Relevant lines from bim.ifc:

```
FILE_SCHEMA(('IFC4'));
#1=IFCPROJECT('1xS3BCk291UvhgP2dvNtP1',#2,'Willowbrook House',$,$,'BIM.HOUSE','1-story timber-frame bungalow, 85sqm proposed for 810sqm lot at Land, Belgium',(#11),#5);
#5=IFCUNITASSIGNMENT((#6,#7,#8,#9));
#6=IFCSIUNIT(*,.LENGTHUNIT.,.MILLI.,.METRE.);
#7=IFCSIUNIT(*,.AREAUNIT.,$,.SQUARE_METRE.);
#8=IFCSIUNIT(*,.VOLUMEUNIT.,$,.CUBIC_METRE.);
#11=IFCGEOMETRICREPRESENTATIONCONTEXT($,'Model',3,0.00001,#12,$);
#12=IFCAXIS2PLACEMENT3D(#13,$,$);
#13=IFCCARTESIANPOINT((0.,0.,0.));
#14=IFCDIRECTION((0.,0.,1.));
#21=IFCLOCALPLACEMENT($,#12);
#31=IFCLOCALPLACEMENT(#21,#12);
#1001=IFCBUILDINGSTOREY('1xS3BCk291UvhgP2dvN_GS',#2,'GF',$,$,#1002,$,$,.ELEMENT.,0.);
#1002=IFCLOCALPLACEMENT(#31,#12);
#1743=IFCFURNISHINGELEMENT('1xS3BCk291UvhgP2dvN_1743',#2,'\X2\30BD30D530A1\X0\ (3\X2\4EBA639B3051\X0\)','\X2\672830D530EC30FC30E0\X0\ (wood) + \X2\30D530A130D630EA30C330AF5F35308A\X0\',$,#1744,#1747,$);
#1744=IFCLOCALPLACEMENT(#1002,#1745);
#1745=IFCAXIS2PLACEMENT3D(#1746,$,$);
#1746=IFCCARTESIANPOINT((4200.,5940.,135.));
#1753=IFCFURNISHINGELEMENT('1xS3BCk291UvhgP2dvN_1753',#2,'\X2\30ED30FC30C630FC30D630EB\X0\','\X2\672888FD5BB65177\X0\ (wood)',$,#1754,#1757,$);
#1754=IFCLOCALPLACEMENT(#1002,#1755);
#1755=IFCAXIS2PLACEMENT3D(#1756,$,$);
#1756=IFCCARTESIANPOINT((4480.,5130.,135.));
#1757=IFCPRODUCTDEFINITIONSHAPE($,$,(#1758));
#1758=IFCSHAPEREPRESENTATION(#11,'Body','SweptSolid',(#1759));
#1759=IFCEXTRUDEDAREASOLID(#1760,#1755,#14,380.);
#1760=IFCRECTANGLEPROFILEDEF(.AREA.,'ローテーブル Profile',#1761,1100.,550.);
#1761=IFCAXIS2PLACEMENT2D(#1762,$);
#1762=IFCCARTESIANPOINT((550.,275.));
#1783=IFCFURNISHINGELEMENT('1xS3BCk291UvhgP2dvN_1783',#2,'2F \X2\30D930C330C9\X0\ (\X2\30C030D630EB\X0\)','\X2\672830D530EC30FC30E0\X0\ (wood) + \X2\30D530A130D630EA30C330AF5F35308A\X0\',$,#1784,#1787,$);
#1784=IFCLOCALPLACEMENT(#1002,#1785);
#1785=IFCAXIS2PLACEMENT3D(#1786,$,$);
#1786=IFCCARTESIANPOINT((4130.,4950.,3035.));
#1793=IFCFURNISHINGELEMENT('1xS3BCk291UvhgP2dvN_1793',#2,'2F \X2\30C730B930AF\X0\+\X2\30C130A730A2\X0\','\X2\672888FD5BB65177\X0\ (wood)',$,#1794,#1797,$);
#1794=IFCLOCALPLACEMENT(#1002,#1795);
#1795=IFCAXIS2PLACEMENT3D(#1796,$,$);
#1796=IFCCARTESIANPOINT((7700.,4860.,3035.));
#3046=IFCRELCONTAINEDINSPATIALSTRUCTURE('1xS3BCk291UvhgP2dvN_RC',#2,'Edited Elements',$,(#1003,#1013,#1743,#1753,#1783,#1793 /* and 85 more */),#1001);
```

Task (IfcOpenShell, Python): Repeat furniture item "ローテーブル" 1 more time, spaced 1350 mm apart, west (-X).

```python
import numpy as np
import ifcopenshell
import ifcopenshell.api.geometry
import ifcopenshell.api.root
import ifcopenshell.util.element
import ifcopenshell.util.placement
import ifcopenshell.util.unit

model = ifcopenshell.open("bim.ifc")
unit_scale = ifcopenshell.util.unit.calculate_unit_scale(model)


def reuse_history(source, copy):
    """copy_class also copies each property set's owner history, people and application; keep the originals."""
    for rel in copy.IsDefinedBy:
        if rel.is_a("IfcRelDefinesByProperties") and (history := rel.RelatingPropertyDefinition.OwnerHistory):
            rel.RelatingPropertyDefinition.OwnerHistory = source.OwnerHistory
            ifcopenshell.util.element.remove_deep2(model, history)


source = model.by_id(1753)
base = ifcopenshell.util.placement.get_local_placement(source.ObjectPlacement)
step = np.array([-1.0, 0.0, 0.0]) * 1.35 / unit_scale

for i in range(1, 2):
    copy = ifcopenshell.api.root.copy_class(model, product=source)
    copy.Representation = ifcopenshell.util.element.copy_deep(
        model, source.Representation, exclude=["IfcGeometricRepresentationContext", "IfcRepresentationMap"]
    )
    reuse_history(source, copy)
    matrix = base.copy()
    matrix[:3, 3] += i * step
    print("added at", matrix[:3, 3].round(3) + 0.0)
    ifcopenshell.api.geometry.edit_object_placement(model, product=copy, matrix=matrix, is_si=False)

model.write("bim_edited.ifc")
```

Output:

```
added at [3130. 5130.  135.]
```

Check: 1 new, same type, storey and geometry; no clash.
